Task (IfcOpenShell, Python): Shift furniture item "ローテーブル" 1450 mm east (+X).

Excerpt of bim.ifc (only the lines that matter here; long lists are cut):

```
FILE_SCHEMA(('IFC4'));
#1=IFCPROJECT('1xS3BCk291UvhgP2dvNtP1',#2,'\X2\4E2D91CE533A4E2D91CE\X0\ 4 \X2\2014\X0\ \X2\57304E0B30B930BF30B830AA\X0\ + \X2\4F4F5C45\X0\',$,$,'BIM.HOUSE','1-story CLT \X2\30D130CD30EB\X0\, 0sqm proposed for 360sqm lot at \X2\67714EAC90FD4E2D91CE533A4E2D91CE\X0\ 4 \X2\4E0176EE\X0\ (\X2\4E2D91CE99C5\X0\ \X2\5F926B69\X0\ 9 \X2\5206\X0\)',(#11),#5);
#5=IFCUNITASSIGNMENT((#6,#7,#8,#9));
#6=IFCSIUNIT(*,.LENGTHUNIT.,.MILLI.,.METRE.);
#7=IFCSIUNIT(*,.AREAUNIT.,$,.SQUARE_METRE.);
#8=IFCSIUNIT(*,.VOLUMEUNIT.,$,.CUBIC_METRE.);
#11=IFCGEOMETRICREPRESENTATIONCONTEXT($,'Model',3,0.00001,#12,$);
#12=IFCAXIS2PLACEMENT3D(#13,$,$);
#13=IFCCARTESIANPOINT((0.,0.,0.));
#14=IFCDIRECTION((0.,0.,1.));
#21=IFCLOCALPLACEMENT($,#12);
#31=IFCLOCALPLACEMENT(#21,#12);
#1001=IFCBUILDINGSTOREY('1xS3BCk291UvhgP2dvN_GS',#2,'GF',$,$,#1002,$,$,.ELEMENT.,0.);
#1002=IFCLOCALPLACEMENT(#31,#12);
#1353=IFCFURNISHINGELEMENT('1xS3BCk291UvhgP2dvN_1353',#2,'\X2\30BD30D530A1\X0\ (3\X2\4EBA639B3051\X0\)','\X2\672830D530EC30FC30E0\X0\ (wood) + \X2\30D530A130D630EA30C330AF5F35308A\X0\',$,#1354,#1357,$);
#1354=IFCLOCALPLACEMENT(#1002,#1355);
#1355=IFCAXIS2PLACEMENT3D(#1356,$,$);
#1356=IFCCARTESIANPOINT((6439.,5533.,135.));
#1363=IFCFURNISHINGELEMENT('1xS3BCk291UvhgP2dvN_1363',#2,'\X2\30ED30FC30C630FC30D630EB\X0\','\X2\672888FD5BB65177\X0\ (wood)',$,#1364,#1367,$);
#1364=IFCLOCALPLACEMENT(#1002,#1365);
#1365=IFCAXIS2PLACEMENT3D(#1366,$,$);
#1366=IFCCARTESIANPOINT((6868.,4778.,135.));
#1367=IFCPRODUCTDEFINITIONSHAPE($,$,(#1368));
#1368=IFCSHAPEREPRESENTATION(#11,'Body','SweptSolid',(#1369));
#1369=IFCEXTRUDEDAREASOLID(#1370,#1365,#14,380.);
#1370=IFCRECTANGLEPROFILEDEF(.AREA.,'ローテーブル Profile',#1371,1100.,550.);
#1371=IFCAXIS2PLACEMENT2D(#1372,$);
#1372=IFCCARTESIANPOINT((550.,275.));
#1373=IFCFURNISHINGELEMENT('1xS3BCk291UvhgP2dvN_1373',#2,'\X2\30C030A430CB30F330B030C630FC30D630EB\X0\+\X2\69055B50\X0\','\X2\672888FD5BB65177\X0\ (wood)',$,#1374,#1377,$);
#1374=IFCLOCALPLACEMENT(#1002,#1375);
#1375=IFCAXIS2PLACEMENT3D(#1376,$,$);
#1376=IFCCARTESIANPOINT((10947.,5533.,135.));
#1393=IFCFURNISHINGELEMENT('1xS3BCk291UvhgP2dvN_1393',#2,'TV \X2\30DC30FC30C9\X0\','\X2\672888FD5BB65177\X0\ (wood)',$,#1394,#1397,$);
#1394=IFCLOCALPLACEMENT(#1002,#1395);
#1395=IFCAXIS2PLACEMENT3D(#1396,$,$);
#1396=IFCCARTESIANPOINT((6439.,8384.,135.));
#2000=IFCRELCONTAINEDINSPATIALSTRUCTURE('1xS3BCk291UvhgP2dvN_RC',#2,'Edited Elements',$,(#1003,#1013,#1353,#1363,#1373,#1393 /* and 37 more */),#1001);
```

```python
import ifcopenshell
import ifcopenshell.api.geometry
import ifcopenshell.util.placement
import ifcopenshell.util.unit

model = ifcopenshell.open("bim.ifc")
unit_scale = ifcopenshell.util.unit.calculate_unit_scale(model)

item = model.by_id(1363)
matrix = ifcopenshell.util.placement.get_local_placement(item.ObjectPlacement)
matrix[0, 3] += 1.45 / unit_scale
ifcopenshell.api.geometry.edit_object_placement(model, product=item, matrix=matrix, is_si=False)

print(ifcopenshell.util.placement.get_local_placement(item.ObjectPlacement).round(3) + 0.0)

model.write("bim_rev.ifc")
```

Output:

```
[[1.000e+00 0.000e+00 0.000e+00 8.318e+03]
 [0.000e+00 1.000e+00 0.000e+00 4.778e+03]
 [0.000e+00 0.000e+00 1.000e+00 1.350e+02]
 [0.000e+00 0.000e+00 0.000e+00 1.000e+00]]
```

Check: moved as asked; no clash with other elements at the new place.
